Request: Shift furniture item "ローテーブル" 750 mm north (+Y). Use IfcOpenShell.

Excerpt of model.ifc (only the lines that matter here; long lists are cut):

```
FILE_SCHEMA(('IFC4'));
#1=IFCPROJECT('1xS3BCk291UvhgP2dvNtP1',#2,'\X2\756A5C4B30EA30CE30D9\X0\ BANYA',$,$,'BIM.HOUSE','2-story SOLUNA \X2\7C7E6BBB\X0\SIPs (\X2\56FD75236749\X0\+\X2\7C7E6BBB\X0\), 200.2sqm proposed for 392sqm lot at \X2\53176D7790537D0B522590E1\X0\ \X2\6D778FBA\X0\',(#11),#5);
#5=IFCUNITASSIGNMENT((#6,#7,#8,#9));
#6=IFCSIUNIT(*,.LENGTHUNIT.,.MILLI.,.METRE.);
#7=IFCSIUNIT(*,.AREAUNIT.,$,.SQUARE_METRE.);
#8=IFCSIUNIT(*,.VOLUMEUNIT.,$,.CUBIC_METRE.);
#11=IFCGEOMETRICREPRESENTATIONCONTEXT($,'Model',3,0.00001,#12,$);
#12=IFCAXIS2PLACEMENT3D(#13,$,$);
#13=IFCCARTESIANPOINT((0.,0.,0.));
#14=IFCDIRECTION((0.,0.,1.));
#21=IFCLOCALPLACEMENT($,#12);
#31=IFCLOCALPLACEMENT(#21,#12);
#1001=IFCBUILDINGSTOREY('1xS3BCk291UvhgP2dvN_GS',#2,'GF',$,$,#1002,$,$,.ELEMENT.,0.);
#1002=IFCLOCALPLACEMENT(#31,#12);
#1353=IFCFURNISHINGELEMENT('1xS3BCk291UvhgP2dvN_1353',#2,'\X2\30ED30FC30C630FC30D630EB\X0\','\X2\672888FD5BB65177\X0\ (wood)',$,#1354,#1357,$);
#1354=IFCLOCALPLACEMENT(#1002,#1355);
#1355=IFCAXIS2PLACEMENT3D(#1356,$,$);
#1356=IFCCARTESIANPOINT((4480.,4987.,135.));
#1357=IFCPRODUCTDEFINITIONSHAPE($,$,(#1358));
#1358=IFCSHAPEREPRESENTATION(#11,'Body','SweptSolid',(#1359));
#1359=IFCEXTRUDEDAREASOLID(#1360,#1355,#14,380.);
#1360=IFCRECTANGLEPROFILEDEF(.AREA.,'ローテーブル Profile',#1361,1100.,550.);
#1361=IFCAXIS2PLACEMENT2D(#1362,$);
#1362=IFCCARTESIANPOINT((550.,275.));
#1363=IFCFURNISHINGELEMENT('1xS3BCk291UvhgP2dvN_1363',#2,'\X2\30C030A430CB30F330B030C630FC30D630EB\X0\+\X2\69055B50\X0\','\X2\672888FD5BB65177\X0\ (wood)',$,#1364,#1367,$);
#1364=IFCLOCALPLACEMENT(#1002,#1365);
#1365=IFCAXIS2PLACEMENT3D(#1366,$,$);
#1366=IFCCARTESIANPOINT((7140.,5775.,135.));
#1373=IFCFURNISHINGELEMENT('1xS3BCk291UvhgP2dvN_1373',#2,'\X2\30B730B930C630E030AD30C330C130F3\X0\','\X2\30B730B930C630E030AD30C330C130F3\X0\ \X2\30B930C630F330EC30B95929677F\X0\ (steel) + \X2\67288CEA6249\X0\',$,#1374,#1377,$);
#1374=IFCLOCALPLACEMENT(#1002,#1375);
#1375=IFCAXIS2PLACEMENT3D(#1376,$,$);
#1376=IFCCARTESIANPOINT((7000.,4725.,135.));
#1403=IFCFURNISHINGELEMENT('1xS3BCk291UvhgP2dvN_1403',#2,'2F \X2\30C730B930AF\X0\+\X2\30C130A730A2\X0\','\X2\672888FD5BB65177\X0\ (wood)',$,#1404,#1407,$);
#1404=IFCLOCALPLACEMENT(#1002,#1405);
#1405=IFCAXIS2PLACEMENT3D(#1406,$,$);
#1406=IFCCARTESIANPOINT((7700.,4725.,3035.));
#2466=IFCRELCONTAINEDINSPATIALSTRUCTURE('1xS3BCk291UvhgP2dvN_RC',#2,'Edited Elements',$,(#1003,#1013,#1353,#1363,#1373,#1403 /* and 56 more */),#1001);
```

```python
import ifcopenshell
import ifcopenshell.api.geometry
import ifcopenshell.util.placement
import ifcopenshell.util.unit

model = ifcopenshell.open("model.ifc")
unit_scale = ifcopenshell.util.unit.calculate_unit_scale(model)

item = model.by_id(1353)
matrix = ifcopenshell.util.placement.get_local_placement(item.ObjectPlacement)
matrix[1, 3] += 0.75 / unit_scale
ifcopenshell.api.geometry.edit_object_placement(model, product=item, matrix=matrix, is_si=False)

print(ifcopenshell.util.placement.get_local_placement(item.ObjectPlacement).round(3) + 0.0)

model.write("model_updated.ifc")
```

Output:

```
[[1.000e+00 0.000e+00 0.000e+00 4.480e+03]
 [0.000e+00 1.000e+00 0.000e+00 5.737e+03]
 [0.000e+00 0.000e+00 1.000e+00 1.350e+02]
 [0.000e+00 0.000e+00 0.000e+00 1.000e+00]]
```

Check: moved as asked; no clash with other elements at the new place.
